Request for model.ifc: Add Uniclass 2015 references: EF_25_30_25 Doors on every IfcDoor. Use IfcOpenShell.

First a look at what the model holds.

```python
import ifcopenshell

model = ifcopenshell.open("model.ifc")
print(model.schema)
print("classifications:", [c.Name for c in model.by_type("IfcClassification")])
for ifc_class in ("IfcDoor", "IfcRoof", "IfcStair", "IfcWall", "IfcWindow"):
    print(ifc_class, len(model.by_type(ifc_class)))
```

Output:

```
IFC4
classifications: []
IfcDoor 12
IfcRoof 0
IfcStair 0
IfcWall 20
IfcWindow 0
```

```python
import ifcopenshell
import ifcopenshell.api.classification

model = ifcopenshell.open("model.ifc")

system = ifcopenshell.api.classification.add_classification(model, classification="Uniclass 2015")

codes = {
    "IfcDoor": ("EF_25_30_25", "Doors"),
}
for ifc_class, (code, name) in codes.items():
    products = model.by_type(ifc_class)
    ifcopenshell.api.classification.add_reference(
        model, products=products, classification=system, identification=code, name=name
    )
    print(code, len(products))

model.write("model-out.ifc")
```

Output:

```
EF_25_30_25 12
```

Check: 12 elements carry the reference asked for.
